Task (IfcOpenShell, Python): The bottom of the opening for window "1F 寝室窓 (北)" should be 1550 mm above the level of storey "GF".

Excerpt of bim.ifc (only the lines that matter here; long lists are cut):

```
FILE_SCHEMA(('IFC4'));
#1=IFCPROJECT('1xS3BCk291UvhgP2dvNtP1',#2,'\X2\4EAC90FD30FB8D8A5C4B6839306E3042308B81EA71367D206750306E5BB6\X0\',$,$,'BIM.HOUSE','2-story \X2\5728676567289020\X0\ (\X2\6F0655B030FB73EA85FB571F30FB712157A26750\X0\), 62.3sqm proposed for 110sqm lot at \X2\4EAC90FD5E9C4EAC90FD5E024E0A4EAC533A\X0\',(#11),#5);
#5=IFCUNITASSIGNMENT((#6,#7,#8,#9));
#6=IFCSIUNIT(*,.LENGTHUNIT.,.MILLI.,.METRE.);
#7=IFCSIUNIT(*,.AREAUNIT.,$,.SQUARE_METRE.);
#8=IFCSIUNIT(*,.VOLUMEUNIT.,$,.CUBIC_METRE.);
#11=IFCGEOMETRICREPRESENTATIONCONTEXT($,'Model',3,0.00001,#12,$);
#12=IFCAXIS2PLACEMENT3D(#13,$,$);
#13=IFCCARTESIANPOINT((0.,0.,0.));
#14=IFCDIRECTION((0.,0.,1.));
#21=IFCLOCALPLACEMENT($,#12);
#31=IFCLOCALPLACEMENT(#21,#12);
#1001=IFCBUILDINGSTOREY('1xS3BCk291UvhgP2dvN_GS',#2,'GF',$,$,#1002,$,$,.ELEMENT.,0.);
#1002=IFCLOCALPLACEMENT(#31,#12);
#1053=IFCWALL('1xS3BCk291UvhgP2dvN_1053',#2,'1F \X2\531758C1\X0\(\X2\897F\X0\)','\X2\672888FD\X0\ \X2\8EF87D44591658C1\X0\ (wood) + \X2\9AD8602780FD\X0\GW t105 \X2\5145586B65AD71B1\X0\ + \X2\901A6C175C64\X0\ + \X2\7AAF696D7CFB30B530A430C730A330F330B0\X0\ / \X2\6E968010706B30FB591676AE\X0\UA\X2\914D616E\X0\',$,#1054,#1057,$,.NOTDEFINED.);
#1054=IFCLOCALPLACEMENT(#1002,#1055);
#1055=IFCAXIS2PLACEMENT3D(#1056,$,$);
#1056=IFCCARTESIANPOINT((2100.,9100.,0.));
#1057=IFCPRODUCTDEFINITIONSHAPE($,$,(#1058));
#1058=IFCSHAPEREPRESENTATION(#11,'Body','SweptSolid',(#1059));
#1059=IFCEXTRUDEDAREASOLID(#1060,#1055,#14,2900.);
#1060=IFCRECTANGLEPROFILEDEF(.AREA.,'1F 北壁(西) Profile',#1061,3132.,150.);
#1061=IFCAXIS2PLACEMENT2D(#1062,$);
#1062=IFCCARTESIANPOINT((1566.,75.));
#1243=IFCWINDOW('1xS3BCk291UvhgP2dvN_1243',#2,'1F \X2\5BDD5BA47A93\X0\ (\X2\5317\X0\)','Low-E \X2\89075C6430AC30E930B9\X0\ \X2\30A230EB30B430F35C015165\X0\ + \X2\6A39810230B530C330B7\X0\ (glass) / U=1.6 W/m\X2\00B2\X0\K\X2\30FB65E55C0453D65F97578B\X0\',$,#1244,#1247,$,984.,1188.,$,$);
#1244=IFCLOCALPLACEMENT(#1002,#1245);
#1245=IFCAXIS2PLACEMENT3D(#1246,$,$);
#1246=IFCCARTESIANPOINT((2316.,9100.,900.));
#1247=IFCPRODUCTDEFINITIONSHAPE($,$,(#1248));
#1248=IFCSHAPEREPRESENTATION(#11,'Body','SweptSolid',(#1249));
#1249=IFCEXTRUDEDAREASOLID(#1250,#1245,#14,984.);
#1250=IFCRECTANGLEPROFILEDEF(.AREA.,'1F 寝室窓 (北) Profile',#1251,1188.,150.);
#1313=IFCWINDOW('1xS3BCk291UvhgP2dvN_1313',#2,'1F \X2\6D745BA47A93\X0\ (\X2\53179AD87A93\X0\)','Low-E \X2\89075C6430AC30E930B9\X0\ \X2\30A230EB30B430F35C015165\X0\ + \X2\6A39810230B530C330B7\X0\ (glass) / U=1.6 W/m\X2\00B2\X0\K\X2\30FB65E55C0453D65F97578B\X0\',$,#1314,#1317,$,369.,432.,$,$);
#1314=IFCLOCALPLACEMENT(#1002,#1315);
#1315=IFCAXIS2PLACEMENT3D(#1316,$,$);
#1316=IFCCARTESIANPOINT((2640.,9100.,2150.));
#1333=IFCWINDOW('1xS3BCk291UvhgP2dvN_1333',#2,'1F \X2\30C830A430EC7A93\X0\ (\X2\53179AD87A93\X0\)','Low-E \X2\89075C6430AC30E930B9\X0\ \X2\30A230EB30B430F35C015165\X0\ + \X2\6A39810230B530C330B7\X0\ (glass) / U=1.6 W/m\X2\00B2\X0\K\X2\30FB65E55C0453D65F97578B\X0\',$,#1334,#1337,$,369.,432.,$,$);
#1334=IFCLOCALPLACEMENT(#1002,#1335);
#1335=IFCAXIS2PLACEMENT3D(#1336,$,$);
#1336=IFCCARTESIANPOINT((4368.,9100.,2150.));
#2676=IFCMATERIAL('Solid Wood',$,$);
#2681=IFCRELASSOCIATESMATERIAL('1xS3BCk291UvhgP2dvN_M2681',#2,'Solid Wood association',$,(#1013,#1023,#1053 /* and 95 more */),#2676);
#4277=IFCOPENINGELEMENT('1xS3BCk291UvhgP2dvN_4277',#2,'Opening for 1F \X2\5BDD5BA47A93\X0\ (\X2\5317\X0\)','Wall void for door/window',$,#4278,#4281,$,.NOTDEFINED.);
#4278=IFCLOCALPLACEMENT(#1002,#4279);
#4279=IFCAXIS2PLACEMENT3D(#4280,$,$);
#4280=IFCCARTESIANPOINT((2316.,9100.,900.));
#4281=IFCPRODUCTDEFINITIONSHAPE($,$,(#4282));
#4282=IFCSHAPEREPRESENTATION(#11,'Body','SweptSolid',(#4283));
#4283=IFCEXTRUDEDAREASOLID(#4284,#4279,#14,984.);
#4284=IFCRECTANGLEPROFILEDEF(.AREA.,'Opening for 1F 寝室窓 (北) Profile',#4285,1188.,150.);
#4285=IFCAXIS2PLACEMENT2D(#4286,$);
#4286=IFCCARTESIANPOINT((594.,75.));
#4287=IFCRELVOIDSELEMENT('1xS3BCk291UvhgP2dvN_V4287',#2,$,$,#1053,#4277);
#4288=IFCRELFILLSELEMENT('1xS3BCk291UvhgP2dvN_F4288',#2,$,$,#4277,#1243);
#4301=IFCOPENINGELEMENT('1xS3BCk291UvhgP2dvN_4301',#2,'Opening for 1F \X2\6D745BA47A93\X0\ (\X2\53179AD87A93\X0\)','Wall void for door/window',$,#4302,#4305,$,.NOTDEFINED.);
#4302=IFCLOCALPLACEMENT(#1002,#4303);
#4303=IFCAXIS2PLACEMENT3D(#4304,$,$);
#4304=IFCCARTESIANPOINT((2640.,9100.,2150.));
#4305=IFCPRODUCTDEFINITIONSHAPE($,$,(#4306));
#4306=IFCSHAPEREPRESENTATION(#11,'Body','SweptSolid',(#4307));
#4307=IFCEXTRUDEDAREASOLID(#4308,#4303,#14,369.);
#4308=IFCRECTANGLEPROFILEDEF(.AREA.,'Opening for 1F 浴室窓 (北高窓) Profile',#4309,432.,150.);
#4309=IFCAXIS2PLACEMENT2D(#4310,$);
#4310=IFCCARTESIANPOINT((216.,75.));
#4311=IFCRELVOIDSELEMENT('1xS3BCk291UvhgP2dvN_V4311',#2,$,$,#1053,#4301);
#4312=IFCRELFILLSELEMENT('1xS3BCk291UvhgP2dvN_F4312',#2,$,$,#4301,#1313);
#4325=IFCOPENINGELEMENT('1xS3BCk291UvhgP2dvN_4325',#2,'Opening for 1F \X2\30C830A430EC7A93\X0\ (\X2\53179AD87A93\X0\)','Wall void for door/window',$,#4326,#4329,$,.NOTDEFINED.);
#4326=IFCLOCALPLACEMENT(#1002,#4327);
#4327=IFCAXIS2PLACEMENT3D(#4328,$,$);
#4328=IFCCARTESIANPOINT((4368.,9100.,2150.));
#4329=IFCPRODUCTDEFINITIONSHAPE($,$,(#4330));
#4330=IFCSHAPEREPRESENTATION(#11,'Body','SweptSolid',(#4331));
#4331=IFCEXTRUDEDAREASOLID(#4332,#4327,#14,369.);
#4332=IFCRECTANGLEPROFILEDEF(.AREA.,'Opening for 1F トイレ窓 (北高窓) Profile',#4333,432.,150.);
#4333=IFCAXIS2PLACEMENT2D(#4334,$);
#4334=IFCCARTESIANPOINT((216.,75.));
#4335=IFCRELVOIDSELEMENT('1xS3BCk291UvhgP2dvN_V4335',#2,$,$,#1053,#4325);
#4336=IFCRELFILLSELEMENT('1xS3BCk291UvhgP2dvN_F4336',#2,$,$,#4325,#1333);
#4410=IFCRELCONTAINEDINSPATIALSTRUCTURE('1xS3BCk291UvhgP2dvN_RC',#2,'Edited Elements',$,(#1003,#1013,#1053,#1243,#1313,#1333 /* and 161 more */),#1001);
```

```python
import numpy as np
import ifcopenshell
import ifcopenshell.api.geometry
import ifcopenshell.geom
import ifcopenshell.util.element
import ifcopenshell.util.placement
import ifcopenshell.util.shape
import ifcopenshell.util.unit

model = ifcopenshell.open("bim.ifc")
unit_scale = ifcopenshell.util.unit.calculate_unit_scale(model)

window = model.by_id(1243)
opening = window.FillsVoids[0].RelatingOpeningElement
storey = ifcopenshell.util.element.get_container(window, ifc_class="IfcBuildingStorey")
level = ifcopenshell.util.placement.get_local_placement(storey.ObjectPlacement)[2, 3]

# The opening's origin need not be at the sill, so measure its lowest point.
shape = ifcopenshell.geom.create_shape(ifcopenshell.geom.settings(), opening)
bottom = ifcopenshell.util.shape.get_shape_bottom_elevation(shape, shape.geometry) / unit_scale
dz = level + 1.55 / unit_scale - bottom

shift = np.array([0.0, 0.0, dz])
# The window is not placed relative to its opening, so move both.
for product in (opening, window):
    matrix = ifcopenshell.util.placement.get_local_placement(product.ObjectPlacement)
    matrix[:3, 3] += shift
    ifcopenshell.api.geometry.edit_object_placement(model, product=product, matrix=matrix, is_si=False)

print(f"moved by {dz * unit_scale:+.3f} m")

model.write("bim_rev.ifc")
```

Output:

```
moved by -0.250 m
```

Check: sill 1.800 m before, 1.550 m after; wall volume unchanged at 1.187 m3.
